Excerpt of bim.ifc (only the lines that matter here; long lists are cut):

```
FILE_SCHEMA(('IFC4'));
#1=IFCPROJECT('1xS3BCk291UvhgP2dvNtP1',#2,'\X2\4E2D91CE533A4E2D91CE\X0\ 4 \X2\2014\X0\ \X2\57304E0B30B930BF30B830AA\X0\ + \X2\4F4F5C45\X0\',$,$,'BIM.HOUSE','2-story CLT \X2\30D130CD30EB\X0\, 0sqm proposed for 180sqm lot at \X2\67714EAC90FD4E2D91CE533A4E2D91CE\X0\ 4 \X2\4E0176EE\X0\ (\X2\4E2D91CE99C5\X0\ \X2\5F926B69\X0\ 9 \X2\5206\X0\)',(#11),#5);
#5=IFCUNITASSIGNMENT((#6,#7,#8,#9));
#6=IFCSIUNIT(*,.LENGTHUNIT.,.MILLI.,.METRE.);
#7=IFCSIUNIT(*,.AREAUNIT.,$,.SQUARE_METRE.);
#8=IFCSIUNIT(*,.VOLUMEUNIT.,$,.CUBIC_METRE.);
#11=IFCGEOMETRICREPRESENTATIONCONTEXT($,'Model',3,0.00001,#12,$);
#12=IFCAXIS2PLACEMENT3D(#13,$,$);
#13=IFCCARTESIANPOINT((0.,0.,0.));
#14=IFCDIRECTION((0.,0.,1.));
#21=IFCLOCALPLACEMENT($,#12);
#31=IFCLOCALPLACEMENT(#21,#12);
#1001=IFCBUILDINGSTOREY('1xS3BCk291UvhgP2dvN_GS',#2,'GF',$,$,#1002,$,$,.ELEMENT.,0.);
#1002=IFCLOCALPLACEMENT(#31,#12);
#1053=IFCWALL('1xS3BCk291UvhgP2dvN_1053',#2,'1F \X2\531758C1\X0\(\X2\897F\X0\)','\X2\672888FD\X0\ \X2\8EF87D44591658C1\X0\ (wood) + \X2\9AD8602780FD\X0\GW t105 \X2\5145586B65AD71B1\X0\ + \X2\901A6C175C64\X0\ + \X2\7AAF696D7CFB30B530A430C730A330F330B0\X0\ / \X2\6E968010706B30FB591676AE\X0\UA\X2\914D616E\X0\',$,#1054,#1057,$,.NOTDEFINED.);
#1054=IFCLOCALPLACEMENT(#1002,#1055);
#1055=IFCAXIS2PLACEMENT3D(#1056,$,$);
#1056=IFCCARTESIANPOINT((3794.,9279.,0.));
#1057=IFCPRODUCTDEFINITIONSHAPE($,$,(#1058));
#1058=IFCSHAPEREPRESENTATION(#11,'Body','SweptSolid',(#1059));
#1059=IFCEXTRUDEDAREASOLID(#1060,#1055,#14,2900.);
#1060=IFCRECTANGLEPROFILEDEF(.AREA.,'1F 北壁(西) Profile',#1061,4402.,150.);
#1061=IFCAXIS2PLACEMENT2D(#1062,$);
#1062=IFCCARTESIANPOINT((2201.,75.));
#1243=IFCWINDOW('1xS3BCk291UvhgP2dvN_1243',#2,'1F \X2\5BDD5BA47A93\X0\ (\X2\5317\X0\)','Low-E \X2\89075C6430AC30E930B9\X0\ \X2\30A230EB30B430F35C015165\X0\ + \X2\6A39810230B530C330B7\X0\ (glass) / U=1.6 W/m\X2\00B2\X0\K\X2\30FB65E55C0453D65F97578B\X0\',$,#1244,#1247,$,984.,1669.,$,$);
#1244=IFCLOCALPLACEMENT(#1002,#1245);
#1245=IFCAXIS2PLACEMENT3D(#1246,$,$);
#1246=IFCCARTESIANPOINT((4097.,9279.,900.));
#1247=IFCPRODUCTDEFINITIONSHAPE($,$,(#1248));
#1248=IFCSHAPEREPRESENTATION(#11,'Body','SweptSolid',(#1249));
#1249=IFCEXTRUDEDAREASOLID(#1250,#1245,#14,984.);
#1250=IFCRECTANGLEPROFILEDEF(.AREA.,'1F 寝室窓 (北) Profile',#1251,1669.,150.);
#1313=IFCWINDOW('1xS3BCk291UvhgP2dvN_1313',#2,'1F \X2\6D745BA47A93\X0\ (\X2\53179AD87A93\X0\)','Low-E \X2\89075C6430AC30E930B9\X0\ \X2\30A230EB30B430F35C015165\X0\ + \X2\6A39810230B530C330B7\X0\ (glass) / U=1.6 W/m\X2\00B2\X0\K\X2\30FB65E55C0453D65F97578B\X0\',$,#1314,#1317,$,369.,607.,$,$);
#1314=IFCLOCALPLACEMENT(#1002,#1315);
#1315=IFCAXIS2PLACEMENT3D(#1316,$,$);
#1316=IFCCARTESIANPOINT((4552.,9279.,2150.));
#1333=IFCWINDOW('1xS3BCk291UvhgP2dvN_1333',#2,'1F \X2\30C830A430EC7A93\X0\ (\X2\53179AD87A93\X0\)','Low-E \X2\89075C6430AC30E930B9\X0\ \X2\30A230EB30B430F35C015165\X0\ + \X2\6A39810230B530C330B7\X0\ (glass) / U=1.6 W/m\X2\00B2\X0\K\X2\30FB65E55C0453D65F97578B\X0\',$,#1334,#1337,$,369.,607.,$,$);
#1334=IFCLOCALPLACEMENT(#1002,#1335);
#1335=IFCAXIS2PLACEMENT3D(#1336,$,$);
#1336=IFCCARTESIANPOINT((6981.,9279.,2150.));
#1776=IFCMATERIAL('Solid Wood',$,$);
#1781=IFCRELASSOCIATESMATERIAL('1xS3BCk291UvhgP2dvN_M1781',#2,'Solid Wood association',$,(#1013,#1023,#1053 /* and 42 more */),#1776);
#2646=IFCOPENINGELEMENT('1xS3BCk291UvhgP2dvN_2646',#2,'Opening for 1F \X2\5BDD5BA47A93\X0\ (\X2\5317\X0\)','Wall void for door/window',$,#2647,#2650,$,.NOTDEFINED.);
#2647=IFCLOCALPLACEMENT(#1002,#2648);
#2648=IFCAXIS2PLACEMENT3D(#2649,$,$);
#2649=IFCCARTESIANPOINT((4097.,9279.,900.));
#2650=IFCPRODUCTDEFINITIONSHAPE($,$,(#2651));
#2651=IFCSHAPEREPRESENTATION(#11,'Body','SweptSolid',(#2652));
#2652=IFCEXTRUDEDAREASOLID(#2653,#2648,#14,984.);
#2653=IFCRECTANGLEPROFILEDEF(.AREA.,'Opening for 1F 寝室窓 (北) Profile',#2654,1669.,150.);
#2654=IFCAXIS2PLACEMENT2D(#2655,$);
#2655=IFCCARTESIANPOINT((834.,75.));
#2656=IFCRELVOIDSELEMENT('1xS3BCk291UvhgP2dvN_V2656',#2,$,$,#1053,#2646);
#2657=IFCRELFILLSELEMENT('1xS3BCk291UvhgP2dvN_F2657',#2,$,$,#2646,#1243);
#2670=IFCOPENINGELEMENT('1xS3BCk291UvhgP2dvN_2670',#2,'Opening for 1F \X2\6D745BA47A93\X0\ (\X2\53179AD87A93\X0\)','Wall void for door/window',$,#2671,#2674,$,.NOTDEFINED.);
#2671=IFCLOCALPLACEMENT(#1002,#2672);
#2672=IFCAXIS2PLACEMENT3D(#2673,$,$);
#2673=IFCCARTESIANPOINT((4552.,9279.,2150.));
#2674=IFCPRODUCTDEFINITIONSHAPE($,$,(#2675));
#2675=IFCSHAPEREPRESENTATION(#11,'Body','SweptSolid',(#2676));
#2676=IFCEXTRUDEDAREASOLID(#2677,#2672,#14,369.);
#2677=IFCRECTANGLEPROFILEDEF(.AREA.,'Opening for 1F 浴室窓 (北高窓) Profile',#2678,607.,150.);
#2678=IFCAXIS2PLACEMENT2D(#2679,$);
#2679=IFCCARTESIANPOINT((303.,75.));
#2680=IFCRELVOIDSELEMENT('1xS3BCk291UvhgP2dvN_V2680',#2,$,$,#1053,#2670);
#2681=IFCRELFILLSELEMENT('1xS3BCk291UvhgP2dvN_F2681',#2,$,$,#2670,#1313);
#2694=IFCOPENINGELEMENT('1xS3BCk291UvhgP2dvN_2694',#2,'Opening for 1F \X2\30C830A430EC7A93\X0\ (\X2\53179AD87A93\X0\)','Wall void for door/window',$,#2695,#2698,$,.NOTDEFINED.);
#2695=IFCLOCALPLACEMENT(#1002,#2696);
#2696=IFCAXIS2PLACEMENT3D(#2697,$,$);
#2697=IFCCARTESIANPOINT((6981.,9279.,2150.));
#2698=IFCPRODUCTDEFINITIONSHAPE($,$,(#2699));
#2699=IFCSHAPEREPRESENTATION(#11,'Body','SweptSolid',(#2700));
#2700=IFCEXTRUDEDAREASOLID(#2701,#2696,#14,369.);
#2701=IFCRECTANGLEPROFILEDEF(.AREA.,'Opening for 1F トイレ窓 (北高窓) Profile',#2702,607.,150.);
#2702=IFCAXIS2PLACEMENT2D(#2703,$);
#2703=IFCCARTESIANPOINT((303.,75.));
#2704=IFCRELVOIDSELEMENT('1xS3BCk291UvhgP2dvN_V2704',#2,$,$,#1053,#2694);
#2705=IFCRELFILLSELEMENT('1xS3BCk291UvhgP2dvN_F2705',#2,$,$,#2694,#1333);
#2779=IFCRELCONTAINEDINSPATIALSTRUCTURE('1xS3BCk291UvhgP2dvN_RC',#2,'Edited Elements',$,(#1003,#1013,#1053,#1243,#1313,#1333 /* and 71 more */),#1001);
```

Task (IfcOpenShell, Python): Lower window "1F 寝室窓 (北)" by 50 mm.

```python
import numpy as np
import ifcopenshell
import ifcopenshell.api.geometry
import ifcopenshell.util.placement
import ifcopenshell.util.unit

model = ifcopenshell.open("bim.ifc")
unit_scale = ifcopenshell.util.unit.calculate_unit_scale(model)

window = model.by_id(1243)
opening = window.FillsVoids[0].RelatingOpeningElement
dz = -0.05 / unit_scale

shift = np.array([0.0, 0.0, dz])
# The window is not placed relative to its opening, so move both.
for product in (opening, window):
    matrix = ifcopenshell.util.placement.get_local_placement(product.ObjectPlacement)
    matrix[:3, 3] += shift
    ifcopenshell.api.geometry.edit_object_placement(model, product=product, matrix=matrix, is_si=False)

print(f"moved by {dz * unit_scale:+.3f} m")

model.write("bim_edited.ifc")
```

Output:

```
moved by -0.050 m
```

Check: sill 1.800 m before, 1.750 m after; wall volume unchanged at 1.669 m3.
